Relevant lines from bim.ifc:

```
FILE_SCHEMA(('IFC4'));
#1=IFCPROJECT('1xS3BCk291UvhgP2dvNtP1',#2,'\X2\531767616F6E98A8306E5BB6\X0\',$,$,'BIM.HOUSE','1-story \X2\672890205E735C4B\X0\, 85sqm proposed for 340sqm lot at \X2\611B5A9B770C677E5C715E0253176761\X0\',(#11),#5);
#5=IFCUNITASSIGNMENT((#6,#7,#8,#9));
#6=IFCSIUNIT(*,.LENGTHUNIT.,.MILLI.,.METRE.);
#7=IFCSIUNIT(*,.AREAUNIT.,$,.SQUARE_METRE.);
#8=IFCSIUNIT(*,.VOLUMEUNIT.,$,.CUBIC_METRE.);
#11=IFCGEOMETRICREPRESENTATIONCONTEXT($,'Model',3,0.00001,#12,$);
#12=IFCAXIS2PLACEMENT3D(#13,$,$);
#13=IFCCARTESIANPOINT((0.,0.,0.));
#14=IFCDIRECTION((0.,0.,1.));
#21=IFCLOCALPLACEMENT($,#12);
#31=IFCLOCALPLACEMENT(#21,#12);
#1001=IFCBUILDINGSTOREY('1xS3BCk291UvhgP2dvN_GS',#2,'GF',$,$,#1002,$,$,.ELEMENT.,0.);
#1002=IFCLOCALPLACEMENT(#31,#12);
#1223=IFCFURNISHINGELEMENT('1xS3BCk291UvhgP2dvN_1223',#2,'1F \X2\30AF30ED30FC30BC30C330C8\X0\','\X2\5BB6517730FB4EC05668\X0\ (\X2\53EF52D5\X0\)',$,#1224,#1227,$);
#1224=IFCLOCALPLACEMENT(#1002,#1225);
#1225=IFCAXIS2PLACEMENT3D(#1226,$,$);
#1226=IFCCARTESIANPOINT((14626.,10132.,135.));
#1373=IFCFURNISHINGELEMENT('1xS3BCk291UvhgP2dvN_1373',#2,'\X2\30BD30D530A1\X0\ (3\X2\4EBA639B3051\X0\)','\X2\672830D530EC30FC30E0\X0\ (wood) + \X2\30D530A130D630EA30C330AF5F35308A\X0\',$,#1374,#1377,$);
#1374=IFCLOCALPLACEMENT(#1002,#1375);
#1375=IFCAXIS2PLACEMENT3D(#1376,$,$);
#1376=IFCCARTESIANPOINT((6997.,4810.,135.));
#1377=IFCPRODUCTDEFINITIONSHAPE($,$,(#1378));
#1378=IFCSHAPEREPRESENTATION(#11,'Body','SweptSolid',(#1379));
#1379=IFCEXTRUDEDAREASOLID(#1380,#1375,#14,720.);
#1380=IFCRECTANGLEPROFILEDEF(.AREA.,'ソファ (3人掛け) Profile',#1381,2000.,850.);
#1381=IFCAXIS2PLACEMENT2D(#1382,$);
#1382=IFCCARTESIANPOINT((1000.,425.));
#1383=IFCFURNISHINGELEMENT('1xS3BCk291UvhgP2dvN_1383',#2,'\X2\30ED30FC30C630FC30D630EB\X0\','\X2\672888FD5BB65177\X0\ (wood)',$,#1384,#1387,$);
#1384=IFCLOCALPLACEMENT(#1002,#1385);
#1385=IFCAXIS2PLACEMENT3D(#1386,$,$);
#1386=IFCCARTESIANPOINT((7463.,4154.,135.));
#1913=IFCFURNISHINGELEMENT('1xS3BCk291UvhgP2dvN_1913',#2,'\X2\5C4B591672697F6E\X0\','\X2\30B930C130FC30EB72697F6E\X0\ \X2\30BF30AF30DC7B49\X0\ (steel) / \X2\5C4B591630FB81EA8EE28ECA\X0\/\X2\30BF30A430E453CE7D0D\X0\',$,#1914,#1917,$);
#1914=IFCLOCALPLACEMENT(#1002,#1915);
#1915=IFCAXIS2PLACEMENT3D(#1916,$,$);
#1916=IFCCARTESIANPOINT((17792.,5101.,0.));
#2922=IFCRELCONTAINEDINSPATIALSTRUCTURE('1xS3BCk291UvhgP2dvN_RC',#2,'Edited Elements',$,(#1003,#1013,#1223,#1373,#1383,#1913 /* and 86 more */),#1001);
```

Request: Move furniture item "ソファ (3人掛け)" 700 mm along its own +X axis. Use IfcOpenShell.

```python
import ifcopenshell
import ifcopenshell.api.geometry
import ifcopenshell.util.placement

model = ifcopenshell.open("bim.ifc")

item = model.by_guid("1xS3BCk291UvhgP2dvN_1373")
matrix = ifcopenshell.util.placement.get_local_placement(item.ObjectPlacement)
matrix[:3, 3] += matrix[:3, 0] * 700.0
ifcopenshell.api.geometry.edit_object_placement(model, product=item, matrix=matrix, is_si=False)

print(ifcopenshell.util.placement.get_local_placement(item.ObjectPlacement).round(3) + 0.0)

model.write("bim_updated.ifc")
```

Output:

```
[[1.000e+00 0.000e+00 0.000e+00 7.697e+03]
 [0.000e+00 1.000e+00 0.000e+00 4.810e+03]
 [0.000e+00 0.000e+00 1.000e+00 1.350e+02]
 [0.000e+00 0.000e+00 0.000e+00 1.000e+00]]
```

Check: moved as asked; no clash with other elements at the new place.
